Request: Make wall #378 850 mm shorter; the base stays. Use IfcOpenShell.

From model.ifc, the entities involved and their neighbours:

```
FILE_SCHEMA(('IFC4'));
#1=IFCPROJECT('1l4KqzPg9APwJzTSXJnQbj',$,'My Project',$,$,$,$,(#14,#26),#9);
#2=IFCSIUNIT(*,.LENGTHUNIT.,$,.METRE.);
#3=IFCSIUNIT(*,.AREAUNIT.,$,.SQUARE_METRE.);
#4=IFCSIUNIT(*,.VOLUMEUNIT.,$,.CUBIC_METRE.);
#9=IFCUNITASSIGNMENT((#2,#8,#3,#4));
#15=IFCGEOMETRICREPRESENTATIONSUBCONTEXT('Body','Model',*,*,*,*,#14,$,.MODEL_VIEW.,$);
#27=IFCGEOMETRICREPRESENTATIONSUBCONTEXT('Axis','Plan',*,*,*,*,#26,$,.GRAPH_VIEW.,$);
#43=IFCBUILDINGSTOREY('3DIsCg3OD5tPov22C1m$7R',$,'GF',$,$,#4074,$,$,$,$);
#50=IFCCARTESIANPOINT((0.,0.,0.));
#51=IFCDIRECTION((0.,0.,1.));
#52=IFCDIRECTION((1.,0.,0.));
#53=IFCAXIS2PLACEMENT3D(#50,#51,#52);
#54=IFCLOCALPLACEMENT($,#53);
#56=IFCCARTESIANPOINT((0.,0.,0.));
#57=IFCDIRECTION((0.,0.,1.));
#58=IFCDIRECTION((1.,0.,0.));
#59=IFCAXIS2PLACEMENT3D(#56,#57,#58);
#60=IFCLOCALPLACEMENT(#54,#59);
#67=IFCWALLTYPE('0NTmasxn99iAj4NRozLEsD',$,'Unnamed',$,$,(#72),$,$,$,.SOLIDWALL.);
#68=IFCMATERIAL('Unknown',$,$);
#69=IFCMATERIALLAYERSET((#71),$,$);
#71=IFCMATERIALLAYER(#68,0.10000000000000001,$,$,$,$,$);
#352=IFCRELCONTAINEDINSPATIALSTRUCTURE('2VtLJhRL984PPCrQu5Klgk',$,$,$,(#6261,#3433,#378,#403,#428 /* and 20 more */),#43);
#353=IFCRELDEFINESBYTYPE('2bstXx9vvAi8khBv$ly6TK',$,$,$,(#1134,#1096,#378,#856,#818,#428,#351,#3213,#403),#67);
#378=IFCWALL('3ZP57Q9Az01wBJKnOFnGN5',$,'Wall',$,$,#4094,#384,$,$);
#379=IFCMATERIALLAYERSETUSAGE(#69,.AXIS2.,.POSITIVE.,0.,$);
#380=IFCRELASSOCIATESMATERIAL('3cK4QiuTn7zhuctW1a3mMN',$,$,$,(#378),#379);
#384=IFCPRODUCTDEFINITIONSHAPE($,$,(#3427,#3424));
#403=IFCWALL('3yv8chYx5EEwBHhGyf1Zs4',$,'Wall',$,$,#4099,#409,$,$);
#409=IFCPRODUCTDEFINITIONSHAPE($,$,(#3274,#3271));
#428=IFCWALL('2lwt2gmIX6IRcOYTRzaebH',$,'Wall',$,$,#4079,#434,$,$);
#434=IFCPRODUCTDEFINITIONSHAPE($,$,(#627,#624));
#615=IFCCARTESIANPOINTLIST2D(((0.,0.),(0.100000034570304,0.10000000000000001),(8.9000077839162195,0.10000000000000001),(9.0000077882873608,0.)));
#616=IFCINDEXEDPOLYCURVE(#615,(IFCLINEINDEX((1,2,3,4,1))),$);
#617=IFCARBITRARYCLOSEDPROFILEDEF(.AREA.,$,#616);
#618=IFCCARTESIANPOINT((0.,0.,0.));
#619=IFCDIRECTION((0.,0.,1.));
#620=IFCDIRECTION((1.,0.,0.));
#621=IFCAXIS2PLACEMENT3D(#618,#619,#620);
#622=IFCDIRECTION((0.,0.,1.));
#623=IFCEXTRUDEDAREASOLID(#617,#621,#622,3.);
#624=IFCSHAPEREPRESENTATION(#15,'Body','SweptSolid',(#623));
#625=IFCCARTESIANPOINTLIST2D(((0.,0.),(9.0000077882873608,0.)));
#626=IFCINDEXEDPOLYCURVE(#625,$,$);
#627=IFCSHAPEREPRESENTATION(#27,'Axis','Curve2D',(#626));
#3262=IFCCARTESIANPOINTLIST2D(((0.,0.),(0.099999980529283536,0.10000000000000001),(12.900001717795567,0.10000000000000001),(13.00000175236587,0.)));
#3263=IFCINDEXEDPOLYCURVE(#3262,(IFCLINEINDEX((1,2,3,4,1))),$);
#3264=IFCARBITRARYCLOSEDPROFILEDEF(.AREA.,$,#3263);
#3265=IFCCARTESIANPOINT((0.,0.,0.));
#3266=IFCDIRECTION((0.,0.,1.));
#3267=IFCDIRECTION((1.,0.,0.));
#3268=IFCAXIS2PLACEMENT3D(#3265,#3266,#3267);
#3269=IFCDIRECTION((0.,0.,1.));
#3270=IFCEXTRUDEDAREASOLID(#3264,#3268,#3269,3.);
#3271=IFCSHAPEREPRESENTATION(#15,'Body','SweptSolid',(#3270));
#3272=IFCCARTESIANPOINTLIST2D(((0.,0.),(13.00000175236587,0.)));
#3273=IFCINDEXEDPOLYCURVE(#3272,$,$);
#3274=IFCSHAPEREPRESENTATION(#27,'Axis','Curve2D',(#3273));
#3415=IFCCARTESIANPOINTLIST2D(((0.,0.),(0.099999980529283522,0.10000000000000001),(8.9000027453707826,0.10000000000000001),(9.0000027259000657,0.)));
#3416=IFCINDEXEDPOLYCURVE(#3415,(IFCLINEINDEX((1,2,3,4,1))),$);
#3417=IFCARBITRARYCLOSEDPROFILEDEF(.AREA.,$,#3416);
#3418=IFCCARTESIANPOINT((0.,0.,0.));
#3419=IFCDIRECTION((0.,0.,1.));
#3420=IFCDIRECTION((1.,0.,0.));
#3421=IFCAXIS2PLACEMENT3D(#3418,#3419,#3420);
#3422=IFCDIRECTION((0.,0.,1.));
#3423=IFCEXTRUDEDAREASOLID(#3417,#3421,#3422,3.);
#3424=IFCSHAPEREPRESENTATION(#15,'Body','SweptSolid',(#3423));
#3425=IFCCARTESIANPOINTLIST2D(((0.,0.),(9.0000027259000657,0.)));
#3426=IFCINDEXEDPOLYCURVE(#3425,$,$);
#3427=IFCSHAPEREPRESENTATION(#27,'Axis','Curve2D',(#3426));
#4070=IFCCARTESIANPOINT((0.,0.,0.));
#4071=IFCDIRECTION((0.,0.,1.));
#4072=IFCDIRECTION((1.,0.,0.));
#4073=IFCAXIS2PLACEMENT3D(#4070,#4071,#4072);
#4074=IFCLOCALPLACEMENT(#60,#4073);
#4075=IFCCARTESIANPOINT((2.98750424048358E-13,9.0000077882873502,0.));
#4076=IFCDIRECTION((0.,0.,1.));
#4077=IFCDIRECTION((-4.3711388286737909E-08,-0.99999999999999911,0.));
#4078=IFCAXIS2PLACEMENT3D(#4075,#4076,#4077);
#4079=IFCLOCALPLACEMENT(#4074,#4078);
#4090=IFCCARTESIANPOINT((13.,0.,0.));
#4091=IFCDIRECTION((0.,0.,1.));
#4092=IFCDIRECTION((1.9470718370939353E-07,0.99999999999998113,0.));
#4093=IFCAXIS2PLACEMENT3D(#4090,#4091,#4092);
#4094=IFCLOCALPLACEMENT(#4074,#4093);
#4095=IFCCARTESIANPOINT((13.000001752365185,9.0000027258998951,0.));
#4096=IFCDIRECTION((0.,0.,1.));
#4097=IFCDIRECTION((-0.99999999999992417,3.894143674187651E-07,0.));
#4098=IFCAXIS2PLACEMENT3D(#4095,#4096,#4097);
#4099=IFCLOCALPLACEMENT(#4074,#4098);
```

```python
import ifcopenshell
import ifcopenshell.geom
import ifcopenshell.util.representation
import ifcopenshell.util.shape
import ifcopenshell.util.unit

model = ifcopenshell.open("model.ifc")
unit_scale = ifcopenshell.util.unit.calculate_unit_scale(model)
settings = ifcopenshell.geom.settings()


def volume(element):
    """Net volume in cubic metres, openings subtracted."""
    shape = ifcopenshell.geom.create_shape(settings, element)
    return ifcopenshell.util.shape.get_volume(shape.geometry)


wall = model.by_guid("3ZP57Q9Az01wBJKnOFnGN5")
before = volume(wall)

body = ifcopenshell.util.representation.get_representation(wall, "Model", "Body")
solid = body.Items[0]
old_height = solid.Depth
solid.Depth -= 0.85 / unit_scale
after = volume(wall)

print(f"height {old_height:g} -> {solid.Depth:g}, volume {before:.3f} -> {after:.3f} m3")

model.write("model_edited.ifc")
```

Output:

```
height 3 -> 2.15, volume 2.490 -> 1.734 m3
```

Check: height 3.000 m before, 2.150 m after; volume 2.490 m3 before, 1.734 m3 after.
